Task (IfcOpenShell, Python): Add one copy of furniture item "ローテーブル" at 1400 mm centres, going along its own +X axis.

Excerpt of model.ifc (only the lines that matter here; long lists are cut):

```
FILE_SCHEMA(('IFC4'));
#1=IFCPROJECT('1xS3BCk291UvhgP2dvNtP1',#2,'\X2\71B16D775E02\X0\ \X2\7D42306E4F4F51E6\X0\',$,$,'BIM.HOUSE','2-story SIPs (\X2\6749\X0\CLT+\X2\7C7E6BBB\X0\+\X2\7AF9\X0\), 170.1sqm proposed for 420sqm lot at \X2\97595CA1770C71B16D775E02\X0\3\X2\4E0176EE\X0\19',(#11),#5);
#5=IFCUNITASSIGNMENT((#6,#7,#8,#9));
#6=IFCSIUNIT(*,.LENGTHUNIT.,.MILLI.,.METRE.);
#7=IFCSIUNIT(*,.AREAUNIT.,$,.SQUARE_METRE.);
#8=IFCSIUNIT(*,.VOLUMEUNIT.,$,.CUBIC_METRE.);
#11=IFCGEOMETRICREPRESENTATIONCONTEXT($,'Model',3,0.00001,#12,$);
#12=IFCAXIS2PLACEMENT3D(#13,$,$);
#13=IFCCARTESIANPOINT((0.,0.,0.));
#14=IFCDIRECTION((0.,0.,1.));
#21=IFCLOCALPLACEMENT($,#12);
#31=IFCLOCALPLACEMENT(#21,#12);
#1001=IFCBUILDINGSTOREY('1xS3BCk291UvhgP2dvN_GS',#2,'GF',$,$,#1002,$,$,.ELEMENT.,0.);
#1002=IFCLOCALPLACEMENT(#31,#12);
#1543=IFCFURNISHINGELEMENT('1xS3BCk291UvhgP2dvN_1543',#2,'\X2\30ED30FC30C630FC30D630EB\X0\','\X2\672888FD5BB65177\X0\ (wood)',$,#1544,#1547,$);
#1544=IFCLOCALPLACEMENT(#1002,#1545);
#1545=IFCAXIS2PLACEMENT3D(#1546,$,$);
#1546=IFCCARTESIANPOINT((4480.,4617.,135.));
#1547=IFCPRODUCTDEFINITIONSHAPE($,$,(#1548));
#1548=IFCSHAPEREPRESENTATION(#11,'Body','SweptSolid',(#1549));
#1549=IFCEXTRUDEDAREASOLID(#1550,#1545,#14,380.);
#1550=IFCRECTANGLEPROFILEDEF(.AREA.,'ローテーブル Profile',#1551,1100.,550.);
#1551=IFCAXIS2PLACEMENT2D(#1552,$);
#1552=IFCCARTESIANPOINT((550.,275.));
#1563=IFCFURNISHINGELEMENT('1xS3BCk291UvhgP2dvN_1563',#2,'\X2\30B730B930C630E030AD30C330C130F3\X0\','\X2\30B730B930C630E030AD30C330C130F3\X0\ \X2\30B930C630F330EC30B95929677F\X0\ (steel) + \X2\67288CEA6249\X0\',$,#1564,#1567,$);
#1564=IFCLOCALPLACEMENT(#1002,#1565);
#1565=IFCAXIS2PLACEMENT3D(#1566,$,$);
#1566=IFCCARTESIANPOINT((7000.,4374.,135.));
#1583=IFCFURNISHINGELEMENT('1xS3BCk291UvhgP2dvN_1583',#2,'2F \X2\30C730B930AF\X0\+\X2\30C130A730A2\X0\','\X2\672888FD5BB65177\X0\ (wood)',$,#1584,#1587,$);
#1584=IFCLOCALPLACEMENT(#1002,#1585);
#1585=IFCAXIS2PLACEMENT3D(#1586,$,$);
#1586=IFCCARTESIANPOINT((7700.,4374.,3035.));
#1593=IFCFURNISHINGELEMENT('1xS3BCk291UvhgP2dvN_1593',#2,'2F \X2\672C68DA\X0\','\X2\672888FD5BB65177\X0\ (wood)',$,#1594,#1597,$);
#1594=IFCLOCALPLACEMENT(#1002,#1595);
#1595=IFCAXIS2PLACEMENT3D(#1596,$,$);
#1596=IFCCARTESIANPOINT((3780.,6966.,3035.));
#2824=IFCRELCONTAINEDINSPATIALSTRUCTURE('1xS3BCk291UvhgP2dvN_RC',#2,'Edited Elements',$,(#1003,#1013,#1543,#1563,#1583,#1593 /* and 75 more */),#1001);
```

```python
import ifcopenshell
import ifcopenshell.api.geometry
import ifcopenshell.api.root
import ifcopenshell.util.element
import ifcopenshell.util.placement

model = ifcopenshell.open("model.ifc")


def reuse_history(source, copy):
    """copy_class also copies each property set's owner history, people and application; keep the originals."""
    for rel in copy.IsDefinedBy:
        if rel.is_a("IfcRelDefinesByProperties") and (history := rel.RelatingPropertyDefinition.OwnerHistory):
            rel.RelatingPropertyDefinition.OwnerHistory = source.OwnerHistory
            ifcopenshell.util.element.remove_deep2(model, history)


source = model.by_guid("1xS3BCk291UvhgP2dvN_1543")
base = ifcopenshell.util.placement.get_local_placement(source.ObjectPlacement)
step = base[:3, 0] * 1400.0

for i in range(1, 2):
    copy = ifcopenshell.api.root.copy_class(model, product=source)
    copy.Representation = ifcopenshell.util.element.copy_deep(
        model, source.Representation, exclude=["IfcGeometricRepresentationContext", "IfcRepresentationMap"]
    )
    reuse_history(source, copy)
    matrix = base.copy()
    matrix[:3, 3] += i * step
    print("added at", matrix[:3, 3].round(3) + 0.0)
    ifcopenshell.api.geometry.edit_object_placement(model, product=copy, matrix=matrix, is_si=False)

model.write("model_edited.ifc")
```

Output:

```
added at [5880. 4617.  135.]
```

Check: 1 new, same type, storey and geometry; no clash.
